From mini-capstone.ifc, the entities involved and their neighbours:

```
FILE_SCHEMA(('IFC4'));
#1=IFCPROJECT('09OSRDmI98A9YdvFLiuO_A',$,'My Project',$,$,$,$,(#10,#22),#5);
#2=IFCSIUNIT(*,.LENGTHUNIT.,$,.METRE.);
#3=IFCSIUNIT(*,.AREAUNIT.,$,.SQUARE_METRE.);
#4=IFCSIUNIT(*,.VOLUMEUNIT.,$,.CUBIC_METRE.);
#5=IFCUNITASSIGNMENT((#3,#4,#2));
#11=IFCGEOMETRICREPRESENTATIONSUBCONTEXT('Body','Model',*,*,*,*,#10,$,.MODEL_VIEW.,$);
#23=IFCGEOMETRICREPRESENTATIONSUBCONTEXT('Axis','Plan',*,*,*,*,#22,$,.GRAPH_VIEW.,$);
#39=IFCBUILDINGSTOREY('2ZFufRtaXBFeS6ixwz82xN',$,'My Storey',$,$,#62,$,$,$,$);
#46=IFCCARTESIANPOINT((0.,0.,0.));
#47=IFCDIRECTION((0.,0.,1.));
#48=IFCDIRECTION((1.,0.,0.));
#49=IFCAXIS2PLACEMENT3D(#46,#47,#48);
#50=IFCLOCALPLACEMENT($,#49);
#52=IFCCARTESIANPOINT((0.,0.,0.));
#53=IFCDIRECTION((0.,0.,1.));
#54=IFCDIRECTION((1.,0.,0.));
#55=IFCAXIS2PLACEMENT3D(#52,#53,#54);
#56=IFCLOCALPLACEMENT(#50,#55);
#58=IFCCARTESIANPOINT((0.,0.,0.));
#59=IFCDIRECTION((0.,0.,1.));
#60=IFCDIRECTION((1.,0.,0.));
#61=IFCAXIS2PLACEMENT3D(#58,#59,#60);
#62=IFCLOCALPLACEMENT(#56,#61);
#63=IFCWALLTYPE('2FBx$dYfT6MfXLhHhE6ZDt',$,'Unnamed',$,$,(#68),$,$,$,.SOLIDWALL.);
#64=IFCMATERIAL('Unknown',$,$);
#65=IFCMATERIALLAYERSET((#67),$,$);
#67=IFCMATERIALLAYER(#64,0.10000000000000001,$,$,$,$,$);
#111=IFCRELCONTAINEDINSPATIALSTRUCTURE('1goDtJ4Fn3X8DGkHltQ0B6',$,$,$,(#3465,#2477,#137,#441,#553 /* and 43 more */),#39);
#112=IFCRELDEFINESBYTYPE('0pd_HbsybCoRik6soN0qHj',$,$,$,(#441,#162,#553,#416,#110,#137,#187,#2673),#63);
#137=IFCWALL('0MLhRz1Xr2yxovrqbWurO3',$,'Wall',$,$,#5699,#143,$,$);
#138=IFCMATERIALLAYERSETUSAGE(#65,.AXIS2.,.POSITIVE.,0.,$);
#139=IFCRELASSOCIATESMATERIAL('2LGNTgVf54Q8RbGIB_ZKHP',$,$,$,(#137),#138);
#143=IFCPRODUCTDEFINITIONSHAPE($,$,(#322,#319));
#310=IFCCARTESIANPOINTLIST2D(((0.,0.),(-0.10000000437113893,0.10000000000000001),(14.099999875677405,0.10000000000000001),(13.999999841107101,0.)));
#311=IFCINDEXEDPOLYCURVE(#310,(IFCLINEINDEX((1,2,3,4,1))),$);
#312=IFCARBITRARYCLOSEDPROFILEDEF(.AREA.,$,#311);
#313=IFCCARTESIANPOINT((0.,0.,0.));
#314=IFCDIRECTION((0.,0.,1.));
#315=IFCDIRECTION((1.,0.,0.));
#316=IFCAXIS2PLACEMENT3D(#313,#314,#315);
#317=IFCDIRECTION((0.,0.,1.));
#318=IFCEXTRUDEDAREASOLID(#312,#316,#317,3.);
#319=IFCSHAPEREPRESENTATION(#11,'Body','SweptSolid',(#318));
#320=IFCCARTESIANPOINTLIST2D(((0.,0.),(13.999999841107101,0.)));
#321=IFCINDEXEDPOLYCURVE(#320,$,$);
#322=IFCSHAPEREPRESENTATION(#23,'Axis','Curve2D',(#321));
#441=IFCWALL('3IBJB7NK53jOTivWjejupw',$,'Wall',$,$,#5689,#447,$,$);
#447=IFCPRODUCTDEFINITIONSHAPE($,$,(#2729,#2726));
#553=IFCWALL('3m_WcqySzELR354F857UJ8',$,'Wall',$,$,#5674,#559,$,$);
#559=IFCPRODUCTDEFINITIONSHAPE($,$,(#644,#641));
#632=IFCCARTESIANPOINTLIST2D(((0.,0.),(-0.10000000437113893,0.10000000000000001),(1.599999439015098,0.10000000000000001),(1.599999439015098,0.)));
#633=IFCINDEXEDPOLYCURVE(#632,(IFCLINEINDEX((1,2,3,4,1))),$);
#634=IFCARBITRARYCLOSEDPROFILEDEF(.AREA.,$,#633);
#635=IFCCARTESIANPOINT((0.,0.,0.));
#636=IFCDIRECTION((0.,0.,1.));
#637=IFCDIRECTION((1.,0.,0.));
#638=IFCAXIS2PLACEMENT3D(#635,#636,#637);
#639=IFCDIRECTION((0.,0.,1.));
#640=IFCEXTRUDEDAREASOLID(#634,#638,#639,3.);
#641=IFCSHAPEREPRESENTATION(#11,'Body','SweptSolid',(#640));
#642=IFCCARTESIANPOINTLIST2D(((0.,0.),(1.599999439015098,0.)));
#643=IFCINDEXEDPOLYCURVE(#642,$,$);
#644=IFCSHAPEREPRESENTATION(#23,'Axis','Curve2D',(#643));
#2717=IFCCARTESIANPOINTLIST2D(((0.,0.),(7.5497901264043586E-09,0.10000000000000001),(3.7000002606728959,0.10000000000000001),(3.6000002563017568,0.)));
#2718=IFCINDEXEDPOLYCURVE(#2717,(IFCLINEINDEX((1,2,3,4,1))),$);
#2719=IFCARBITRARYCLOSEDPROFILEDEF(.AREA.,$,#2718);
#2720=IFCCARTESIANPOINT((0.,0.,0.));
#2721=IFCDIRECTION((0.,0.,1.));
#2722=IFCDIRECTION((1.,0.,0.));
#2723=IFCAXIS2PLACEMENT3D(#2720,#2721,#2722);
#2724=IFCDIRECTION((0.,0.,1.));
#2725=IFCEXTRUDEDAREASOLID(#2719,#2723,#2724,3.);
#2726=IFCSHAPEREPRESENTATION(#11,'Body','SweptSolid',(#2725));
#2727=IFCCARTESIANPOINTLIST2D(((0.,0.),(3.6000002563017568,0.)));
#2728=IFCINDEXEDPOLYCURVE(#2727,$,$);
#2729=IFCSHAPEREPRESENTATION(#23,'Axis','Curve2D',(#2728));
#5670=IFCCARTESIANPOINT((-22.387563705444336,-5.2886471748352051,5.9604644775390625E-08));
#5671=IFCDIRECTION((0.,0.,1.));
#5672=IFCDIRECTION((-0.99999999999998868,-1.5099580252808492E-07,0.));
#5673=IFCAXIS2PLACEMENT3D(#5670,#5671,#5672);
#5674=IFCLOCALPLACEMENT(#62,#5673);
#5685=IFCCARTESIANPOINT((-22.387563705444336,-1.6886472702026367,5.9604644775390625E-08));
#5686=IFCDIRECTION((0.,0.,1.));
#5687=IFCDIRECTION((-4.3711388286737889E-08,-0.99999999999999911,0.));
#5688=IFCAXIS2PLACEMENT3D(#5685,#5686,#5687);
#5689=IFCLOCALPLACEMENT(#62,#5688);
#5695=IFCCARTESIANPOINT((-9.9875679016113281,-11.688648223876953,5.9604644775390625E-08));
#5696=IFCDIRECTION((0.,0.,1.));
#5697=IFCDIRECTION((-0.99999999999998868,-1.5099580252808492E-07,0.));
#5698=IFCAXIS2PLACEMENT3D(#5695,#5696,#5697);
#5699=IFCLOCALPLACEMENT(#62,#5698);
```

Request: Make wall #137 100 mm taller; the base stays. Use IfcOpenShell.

```python
import ifcopenshell
import ifcopenshell.geom
import ifcopenshell.util.representation
import ifcopenshell.util.shape
import ifcopenshell.util.unit

model = ifcopenshell.open("mini-capstone.ifc")
unit_scale = ifcopenshell.util.unit.calculate_unit_scale(model)
settings = ifcopenshell.geom.settings()


def volume(element):
    """Net volume in cubic metres, openings subtracted."""
    shape = ifcopenshell.geom.create_shape(settings, element)
    return ifcopenshell.util.shape.get_volume(shape.geometry)


wall = model.by_id(137)
before = volume(wall)

body = ifcopenshell.util.representation.get_representation(wall, "Model", "Body")
solid = body.Items[0]
old_height = solid.Depth
solid.Depth += 0.1 / unit_scale
after = volume(wall)

print(f"height {old_height:g} -> {solid.Depth:g}, volume {before:.3f} -> {after:.3f} m3")

model.write("mini-capstone-out.ifc")
```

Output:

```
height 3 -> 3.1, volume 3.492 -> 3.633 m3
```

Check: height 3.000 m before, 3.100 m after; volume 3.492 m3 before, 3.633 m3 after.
